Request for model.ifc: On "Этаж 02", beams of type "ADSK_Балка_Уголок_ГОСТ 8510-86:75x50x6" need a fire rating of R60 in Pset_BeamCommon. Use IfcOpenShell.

First a look at what the model holds.

```python
import ifcopenshell
import ifcopenshell.util.element

model = ifcopenshell.open("model.ifc")
print(model.schema)
storey = next(s for s in model.by_type("IfcBuildingStorey") if s.Name == "Этаж 02")
beams = [e for e in ifcopenshell.util.element.get_decomposition(storey) if e.is_a("IfcBeam")]
seen = {}
for e in beams:
    element_type = ifcopenshell.util.element.get_type(e)
    key = (element_type.Name if element_type != e and element_type else None, ifcopenshell.util.element.get_pset(e, "Pset_BeamCommon", "FireRating"))
    seen[key] = seen.get(key, 0) + 1
for (name, value), count in sorted(seen.items(), key=str):
    print(count, "x", name, "|", value)
```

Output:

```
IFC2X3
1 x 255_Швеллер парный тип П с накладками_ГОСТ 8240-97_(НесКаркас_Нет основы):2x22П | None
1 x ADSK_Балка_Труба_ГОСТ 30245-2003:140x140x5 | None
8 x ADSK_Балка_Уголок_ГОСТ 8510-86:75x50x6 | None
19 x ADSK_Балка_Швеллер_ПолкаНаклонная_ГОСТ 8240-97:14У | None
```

```python
import ifcopenshell
import ifcopenshell.api.pset
import ifcopenshell.util.element

model = ifcopenshell.open("model.ifc")

storey = next(s for s in model.by_type("IfcBuildingStorey") if s.Name == "Этаж 02")
beams = [e for e in ifcopenshell.util.element.get_decomposition(storey) if e.is_a("IfcBeam")]

count = 0
for e in beams:
    element_type = ifcopenshell.util.element.get_type(e)
    if element_type in (None, e) or element_type.Name != "ADSK_Балка_Уголок_ГОСТ 8510-86:75x50x6":
        continue
    # add_pset returns the element's existing set when there is one.
    pset = ifcopenshell.api.pset.add_pset(model, product=e, name="Pset_BeamCommon")
    ifcopenshell.api.pset.edit_pset(model, pset=pset, properties={"FireRating": "R60"})
    count += 1

print(count, "beams updated")

model.write("model_rev.ifc")
```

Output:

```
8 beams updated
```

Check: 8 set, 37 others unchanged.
